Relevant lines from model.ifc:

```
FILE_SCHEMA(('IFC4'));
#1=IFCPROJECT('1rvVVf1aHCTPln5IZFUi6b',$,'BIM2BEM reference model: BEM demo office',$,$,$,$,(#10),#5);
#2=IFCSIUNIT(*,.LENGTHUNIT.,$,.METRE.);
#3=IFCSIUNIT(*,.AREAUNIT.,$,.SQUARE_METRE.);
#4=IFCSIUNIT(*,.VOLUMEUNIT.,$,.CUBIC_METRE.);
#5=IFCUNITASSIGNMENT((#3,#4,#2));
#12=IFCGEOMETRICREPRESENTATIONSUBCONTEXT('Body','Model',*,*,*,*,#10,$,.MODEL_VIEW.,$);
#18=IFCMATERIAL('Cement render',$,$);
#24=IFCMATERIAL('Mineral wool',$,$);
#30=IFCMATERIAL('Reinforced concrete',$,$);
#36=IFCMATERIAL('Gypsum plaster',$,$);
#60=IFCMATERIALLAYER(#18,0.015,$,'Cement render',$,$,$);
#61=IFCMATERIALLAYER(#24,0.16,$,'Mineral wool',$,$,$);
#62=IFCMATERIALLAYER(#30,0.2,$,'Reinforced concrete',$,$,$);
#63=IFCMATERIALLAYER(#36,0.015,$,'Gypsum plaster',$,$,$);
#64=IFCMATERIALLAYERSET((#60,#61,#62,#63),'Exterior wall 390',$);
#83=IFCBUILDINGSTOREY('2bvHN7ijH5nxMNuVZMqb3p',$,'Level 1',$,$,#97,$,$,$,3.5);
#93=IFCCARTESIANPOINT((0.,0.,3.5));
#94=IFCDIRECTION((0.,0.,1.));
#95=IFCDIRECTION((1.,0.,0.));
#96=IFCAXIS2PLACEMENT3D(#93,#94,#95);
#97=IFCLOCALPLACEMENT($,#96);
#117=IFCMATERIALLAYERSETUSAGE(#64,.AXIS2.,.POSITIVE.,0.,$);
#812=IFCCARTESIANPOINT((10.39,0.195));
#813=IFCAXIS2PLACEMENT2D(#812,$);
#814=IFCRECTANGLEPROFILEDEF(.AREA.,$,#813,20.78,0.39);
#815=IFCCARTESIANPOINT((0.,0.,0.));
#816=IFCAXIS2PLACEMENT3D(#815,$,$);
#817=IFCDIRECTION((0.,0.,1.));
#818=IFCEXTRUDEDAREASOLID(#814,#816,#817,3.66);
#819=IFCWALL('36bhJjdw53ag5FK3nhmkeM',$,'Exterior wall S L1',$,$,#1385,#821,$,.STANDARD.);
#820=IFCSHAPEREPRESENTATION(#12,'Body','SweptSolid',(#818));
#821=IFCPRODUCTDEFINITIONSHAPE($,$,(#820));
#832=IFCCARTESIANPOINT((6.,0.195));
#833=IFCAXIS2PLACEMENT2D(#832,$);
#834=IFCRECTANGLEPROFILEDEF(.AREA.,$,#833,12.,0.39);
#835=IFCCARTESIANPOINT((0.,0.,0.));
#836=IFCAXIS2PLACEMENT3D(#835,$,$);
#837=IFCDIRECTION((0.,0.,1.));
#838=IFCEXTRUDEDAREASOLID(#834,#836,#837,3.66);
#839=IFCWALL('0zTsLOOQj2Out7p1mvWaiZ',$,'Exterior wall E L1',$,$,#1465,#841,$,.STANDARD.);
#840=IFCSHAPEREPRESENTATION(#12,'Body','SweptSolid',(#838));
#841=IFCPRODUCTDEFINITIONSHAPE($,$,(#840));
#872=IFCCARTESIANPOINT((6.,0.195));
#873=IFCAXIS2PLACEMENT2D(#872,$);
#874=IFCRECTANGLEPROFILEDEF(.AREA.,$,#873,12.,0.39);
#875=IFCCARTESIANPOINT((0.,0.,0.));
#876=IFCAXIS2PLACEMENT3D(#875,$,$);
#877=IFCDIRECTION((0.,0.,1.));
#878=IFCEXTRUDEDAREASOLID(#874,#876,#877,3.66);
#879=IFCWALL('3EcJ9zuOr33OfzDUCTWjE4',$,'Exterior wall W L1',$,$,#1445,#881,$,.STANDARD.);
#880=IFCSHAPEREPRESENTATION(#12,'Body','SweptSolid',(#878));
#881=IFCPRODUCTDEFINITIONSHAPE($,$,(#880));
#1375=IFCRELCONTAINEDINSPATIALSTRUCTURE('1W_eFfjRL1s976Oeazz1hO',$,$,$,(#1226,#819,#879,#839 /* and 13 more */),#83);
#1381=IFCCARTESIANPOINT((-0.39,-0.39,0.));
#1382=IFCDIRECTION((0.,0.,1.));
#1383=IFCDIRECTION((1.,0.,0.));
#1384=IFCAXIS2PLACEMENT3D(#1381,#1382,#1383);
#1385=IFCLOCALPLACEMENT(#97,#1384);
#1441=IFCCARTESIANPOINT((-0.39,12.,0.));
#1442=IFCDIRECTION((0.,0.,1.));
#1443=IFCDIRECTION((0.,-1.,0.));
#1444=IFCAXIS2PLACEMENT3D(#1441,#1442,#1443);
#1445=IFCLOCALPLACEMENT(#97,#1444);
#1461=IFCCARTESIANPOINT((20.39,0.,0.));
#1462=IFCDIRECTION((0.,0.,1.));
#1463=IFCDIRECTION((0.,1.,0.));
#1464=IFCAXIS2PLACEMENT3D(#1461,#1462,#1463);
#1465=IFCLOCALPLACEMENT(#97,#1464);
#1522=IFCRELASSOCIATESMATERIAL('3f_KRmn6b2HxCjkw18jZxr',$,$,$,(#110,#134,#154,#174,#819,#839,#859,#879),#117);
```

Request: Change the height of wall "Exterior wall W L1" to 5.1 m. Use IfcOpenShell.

```python
import ifcopenshell
import ifcopenshell.geom
import ifcopenshell.util.representation
import ifcopenshell.util.shape
import ifcopenshell.util.unit

model = ifcopenshell.open("model.ifc")
unit_scale = ifcopenshell.util.unit.calculate_unit_scale(model)
settings = ifcopenshell.geom.settings()


def volume(element):
    """Net volume in cubic metres, openings subtracted."""
    shape = ifcopenshell.geom.create_shape(settings, element)
    return ifcopenshell.util.shape.get_volume(shape.geometry)


wall = model.by_guid("3EcJ9zuOr33OfzDUCTWjE4")
before = volume(wall)

body = ifcopenshell.util.representation.get_representation(wall, "Model", "Body")
solid = body.Items[0]
old_height = solid.Depth
solid.Depth = 5.1 / unit_scale
after = volume(wall)

print(f"height {old_height:g} -> {solid.Depth:g}, volume {before:.3f} -> {after:.3f} m3")

model.write("model-out.ifc")
```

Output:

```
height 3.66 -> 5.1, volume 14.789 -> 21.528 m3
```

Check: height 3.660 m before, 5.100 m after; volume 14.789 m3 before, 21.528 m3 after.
